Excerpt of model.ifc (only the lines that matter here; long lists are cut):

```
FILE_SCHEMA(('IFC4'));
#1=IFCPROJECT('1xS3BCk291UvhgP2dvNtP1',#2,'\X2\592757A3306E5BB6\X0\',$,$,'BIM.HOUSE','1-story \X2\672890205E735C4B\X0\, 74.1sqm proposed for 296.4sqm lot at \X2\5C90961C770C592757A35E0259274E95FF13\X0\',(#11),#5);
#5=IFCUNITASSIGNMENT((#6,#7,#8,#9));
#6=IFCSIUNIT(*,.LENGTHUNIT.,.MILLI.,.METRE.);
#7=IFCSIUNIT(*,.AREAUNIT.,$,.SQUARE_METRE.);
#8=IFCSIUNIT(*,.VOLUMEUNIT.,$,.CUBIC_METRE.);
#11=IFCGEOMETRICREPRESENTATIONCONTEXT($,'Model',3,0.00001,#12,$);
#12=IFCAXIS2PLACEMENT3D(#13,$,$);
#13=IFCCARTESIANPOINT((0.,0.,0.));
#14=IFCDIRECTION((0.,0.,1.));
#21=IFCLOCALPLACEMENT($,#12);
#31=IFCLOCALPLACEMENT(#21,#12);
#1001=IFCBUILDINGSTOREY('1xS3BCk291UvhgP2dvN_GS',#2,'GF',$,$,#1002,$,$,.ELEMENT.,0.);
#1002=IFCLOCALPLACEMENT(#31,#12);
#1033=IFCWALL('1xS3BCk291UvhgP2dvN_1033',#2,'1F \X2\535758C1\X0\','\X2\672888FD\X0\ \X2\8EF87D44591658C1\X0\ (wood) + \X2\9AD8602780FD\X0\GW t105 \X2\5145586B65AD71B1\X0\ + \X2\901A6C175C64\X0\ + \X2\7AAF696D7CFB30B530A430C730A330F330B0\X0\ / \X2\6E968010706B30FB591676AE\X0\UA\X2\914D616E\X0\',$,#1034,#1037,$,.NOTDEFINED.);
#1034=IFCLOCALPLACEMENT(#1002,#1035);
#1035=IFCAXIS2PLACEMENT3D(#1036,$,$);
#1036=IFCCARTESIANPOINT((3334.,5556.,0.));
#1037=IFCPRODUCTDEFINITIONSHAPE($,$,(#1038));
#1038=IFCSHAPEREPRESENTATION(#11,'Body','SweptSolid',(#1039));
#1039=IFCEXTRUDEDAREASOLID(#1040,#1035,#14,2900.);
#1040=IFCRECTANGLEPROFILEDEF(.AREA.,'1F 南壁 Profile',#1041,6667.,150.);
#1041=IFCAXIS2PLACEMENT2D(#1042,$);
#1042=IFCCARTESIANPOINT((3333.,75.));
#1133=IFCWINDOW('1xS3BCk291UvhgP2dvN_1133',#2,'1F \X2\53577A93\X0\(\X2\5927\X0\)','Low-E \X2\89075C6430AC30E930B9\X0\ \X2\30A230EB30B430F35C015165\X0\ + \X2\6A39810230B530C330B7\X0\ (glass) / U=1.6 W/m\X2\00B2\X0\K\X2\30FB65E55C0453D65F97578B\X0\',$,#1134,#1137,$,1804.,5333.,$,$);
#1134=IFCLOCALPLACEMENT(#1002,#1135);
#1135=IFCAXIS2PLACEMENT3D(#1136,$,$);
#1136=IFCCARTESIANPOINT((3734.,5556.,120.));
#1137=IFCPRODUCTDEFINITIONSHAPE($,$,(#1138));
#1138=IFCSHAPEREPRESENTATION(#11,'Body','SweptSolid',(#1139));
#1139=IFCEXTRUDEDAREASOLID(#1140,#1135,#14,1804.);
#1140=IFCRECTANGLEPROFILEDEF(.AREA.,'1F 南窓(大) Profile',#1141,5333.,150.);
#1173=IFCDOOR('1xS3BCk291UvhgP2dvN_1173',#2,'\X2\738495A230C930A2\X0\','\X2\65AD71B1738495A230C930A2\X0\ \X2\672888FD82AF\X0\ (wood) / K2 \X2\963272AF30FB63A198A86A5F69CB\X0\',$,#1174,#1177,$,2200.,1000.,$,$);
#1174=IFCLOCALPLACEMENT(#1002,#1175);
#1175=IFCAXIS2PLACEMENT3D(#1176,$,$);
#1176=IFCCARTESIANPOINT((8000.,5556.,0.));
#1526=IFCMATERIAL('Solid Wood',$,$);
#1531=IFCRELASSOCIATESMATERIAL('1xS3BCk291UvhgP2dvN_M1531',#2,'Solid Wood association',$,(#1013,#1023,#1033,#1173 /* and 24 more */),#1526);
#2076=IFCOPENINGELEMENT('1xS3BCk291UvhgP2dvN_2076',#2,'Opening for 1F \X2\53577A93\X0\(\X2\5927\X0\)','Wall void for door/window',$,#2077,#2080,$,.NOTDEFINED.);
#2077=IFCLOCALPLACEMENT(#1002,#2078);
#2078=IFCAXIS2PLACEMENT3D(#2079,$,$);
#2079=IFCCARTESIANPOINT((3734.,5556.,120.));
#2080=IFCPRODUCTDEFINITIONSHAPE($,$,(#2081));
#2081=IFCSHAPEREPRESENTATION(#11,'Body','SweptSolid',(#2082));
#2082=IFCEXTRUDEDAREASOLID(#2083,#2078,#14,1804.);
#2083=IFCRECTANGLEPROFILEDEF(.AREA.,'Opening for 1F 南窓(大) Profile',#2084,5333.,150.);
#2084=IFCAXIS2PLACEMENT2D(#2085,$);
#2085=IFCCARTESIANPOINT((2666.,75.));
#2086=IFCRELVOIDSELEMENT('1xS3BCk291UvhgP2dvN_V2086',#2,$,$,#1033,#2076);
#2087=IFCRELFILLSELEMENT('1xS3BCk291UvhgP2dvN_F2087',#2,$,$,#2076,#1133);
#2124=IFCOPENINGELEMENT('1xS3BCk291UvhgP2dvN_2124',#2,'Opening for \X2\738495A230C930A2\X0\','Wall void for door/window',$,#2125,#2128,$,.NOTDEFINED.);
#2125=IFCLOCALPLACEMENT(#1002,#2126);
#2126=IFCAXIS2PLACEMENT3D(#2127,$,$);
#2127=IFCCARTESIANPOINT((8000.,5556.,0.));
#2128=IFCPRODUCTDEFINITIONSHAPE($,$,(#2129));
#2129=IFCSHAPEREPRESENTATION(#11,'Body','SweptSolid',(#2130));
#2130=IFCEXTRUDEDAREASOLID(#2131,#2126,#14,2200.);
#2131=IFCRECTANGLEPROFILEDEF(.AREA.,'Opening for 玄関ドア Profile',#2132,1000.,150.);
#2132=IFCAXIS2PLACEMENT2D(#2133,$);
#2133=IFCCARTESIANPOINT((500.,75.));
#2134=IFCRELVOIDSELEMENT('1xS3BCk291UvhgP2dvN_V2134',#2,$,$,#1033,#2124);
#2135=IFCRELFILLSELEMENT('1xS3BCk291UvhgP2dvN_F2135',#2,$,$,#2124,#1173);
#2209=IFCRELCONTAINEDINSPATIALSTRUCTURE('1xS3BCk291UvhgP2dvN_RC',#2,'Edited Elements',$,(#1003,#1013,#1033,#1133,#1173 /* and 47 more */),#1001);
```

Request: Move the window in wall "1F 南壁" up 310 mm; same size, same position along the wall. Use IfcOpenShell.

```python
import numpy as np
import ifcopenshell
import ifcopenshell.api.geometry
import ifcopenshell.util.placement
import ifcopenshell.util.unit

model = ifcopenshell.open("model.ifc")
unit_scale = ifcopenshell.util.unit.calculate_unit_scale(model)

window = model.by_guid("1xS3BCk291UvhgP2dvN_1133")
opening = window.FillsVoids[0].RelatingOpeningElement
dz = 310.0

shift = np.array([0.0, 0.0, dz])
# The window is not placed relative to its opening, so move both.
for product in (opening, window):
    matrix = ifcopenshell.util.placement.get_local_placement(product.ObjectPlacement)
    matrix[:3, 3] += shift
    ifcopenshell.api.geometry.edit_object_placement(model, product=product, matrix=matrix, is_si=False)

print(f"moved by {dz * unit_scale:+.3f} m")

model.write("model_rev.ifc")
```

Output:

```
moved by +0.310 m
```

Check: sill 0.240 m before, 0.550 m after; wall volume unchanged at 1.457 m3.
